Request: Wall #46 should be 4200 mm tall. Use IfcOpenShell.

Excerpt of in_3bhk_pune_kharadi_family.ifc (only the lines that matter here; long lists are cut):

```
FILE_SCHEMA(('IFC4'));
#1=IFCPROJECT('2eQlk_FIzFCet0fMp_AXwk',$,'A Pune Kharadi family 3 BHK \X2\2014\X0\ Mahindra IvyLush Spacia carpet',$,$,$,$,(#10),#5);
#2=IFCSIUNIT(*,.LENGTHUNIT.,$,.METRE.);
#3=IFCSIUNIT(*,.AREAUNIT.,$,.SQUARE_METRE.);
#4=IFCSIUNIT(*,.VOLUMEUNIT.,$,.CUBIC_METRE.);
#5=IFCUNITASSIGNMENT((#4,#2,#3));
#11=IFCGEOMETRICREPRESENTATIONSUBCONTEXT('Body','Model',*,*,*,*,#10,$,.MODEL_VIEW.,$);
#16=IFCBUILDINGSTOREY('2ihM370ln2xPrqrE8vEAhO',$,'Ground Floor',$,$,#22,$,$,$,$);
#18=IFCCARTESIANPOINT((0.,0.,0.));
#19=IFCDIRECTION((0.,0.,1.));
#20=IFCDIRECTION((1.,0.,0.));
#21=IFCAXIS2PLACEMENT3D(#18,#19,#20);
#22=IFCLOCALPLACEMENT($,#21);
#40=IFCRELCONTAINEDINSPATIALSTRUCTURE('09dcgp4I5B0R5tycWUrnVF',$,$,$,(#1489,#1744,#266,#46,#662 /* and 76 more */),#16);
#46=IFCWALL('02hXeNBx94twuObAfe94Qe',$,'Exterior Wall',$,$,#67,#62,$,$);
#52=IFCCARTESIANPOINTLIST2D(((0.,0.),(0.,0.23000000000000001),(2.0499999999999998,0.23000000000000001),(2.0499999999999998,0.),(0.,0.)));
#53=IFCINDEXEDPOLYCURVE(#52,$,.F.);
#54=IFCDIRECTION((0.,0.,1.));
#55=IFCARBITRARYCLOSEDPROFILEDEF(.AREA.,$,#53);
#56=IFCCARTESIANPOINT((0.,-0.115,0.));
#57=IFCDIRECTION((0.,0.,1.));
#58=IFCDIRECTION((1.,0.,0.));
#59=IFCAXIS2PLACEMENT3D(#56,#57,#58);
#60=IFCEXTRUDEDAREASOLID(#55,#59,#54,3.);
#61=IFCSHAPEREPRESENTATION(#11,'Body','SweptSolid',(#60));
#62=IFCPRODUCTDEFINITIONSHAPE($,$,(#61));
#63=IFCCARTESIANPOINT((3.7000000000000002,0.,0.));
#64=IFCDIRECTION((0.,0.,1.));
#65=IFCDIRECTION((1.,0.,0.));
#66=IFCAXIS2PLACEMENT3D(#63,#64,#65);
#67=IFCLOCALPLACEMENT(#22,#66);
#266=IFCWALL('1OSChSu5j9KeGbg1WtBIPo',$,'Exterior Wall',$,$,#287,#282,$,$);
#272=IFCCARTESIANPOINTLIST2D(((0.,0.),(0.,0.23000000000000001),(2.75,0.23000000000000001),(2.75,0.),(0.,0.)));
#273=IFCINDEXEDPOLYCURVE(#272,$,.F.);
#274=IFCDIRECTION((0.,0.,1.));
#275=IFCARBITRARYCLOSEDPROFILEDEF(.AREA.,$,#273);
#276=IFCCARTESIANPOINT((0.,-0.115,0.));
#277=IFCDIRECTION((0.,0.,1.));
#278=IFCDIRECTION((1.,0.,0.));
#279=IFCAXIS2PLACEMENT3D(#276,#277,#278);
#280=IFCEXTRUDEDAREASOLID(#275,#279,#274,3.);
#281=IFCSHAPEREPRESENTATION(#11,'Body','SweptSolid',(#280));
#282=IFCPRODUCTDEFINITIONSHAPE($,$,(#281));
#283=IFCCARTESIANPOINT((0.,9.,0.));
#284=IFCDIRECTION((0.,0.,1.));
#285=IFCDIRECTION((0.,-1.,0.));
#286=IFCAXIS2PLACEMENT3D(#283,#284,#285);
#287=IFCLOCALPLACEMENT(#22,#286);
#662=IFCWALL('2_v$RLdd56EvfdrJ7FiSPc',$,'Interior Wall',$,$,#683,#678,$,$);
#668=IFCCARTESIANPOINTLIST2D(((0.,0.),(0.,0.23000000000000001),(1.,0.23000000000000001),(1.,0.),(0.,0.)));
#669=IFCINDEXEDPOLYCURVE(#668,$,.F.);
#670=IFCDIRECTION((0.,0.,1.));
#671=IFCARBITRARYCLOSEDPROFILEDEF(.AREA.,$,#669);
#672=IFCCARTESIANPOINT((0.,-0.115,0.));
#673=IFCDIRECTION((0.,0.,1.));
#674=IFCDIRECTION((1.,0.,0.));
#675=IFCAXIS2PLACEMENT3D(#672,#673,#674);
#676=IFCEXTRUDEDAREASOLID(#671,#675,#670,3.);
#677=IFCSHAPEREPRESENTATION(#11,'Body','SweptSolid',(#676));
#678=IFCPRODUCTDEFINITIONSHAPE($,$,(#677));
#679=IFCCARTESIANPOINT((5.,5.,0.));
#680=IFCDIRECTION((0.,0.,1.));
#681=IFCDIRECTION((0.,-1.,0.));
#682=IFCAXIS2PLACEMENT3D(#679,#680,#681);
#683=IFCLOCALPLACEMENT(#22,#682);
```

```python
import ifcopenshell
import ifcopenshell.geom
import ifcopenshell.util.representation
import ifcopenshell.util.shape
import ifcopenshell.util.unit

model = ifcopenshell.open("in_3bhk_pune_kharadi_family.ifc")
unit_scale = ifcopenshell.util.unit.calculate_unit_scale(model)
settings = ifcopenshell.geom.settings()


def volume(element):
    """Net volume in cubic metres, openings subtracted."""
    shape = ifcopenshell.geom.create_shape(settings, element)
    return ifcopenshell.util.shape.get_volume(shape.geometry)


wall = model.by_guid("02hXeNBx94twuObAfe94Qe")
before = volume(wall)

body = ifcopenshell.util.representation.get_representation(wall, "Model", "Body")
solid = body.Items[0]
old_height = solid.Depth
solid.Depth = 4.2 / unit_scale
after = volume(wall)

print(f"height {old_height:g} -> {solid.Depth:g}, volume {before:.3f} -> {after:.3f} m3")

model.write("in_3bhk_pune_kharadi_family_updated.ifc")
```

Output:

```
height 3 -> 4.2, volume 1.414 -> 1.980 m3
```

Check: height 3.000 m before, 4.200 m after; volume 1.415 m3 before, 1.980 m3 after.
